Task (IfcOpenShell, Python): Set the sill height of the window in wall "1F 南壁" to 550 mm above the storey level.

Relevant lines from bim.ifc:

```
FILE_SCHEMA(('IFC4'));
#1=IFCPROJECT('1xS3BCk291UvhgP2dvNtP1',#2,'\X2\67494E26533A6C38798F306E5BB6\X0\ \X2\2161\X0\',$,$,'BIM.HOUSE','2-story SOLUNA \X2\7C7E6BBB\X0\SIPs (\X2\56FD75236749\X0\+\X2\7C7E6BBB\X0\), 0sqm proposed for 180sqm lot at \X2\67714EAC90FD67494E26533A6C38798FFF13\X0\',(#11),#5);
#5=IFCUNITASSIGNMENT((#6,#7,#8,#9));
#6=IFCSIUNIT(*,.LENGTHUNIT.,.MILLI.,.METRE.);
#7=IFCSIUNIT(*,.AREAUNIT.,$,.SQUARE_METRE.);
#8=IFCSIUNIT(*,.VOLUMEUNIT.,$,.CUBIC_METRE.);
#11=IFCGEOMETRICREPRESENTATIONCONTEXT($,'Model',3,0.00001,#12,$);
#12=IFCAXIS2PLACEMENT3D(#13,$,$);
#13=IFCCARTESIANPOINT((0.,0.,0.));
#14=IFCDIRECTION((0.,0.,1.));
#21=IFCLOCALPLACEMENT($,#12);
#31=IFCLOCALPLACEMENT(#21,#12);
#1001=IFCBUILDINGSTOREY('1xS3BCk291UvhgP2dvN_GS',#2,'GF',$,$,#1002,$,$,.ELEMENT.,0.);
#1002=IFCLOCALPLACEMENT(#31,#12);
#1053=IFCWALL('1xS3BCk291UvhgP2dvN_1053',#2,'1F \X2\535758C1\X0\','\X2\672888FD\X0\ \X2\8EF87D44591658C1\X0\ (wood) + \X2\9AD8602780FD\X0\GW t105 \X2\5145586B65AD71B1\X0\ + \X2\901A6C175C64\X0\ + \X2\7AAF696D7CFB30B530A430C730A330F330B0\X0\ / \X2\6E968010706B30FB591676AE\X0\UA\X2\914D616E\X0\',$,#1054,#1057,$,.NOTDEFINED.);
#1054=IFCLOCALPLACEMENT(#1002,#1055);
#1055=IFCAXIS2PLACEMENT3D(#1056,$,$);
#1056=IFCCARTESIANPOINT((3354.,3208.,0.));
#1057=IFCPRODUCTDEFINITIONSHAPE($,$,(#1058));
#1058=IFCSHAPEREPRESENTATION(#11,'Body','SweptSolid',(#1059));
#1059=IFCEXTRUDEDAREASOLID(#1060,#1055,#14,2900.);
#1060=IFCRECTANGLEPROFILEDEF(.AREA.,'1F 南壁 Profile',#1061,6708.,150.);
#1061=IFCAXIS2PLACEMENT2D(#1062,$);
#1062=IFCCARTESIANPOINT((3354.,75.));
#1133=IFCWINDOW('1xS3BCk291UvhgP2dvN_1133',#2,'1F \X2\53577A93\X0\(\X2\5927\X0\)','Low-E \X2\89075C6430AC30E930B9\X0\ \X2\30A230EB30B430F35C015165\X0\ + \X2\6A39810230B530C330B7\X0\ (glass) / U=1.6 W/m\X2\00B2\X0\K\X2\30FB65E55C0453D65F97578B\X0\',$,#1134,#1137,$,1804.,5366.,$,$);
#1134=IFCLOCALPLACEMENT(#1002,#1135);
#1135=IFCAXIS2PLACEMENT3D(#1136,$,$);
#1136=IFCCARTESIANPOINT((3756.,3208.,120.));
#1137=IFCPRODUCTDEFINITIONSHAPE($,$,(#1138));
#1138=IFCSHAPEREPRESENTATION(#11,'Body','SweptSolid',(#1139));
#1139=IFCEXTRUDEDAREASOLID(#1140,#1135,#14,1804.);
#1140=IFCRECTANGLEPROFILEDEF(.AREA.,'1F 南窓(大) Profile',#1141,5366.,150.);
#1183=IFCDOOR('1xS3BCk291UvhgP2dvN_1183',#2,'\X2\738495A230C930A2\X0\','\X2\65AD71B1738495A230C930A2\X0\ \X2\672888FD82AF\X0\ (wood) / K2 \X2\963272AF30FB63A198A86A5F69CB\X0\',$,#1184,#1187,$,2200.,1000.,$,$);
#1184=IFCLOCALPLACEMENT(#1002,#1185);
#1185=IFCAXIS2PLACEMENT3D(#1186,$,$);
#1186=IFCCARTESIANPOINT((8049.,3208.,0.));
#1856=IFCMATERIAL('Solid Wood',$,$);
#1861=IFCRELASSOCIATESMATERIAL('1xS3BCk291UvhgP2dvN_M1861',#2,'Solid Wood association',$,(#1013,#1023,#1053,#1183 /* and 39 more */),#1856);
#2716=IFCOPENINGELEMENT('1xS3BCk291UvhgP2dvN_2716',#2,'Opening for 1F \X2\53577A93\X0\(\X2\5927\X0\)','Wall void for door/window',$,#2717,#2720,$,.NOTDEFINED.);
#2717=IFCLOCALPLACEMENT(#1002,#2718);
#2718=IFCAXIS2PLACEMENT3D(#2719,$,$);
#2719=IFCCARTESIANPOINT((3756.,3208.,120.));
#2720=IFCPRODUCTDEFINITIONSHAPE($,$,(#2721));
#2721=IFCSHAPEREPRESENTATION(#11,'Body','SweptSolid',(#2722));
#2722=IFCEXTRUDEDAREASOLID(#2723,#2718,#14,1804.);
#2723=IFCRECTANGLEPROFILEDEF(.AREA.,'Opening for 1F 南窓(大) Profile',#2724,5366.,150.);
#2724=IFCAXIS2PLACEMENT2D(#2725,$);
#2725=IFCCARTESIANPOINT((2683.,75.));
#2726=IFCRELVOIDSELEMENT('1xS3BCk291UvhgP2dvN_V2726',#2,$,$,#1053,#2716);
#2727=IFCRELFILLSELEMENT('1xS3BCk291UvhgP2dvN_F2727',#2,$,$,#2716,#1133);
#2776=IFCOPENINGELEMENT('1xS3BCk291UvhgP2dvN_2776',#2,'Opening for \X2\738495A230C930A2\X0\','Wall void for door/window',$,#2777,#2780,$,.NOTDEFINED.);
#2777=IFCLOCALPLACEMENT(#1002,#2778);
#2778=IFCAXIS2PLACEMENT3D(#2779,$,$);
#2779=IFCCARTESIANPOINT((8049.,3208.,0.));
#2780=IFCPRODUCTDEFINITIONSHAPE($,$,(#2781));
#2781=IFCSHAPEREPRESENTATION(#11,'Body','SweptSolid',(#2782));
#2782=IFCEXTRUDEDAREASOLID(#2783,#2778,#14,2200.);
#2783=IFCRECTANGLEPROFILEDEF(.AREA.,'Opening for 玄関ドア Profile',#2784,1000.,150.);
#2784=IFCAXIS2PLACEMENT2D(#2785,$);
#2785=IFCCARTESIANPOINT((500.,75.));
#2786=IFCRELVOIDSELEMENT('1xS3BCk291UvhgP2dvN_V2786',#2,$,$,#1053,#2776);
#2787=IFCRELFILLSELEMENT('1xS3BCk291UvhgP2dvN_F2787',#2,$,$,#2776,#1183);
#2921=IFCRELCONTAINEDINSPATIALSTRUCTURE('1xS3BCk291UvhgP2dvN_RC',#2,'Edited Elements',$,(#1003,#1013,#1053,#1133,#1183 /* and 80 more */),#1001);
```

```python
import numpy as np
import ifcopenshell
import ifcopenshell.api.geometry
import ifcopenshell.geom
import ifcopenshell.util.element
import ifcopenshell.util.placement
import ifcopenshell.util.shape
import ifcopenshell.util.unit

model = ifcopenshell.open("bim.ifc")
unit_scale = ifcopenshell.util.unit.calculate_unit_scale(model)

window = model.by_guid("1xS3BCk291UvhgP2dvN_1133")
opening = window.FillsVoids[0].RelatingOpeningElement
storey = ifcopenshell.util.element.get_container(window, ifc_class="IfcBuildingStorey")
level = ifcopenshell.util.placement.get_local_placement(storey.ObjectPlacement)[2, 3]

# The opening's origin need not be at the sill, so measure its lowest point.
shape = ifcopenshell.geom.create_shape(ifcopenshell.geom.settings(), opening)
bottom = ifcopenshell.util.shape.get_shape_bottom_elevation(shape, shape.geometry) / unit_scale
dz = level + 0.55 / unit_scale - bottom

shift = np.array([0.0, 0.0, dz])
# The window is not placed relative to its opening, so move both.
for product in (opening, window):
    matrix = ifcopenshell.util.placement.get_local_placement(product.ObjectPlacement)
    matrix[:3, 3] += shift
    ifcopenshell.api.geometry.edit_object_placement(model, product=product, matrix=matrix, is_si=False)

print(f"moved by {dz * unit_scale:+.3f} m")

model.write("bim_rev.ifc")
```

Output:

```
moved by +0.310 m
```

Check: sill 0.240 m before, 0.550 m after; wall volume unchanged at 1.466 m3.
